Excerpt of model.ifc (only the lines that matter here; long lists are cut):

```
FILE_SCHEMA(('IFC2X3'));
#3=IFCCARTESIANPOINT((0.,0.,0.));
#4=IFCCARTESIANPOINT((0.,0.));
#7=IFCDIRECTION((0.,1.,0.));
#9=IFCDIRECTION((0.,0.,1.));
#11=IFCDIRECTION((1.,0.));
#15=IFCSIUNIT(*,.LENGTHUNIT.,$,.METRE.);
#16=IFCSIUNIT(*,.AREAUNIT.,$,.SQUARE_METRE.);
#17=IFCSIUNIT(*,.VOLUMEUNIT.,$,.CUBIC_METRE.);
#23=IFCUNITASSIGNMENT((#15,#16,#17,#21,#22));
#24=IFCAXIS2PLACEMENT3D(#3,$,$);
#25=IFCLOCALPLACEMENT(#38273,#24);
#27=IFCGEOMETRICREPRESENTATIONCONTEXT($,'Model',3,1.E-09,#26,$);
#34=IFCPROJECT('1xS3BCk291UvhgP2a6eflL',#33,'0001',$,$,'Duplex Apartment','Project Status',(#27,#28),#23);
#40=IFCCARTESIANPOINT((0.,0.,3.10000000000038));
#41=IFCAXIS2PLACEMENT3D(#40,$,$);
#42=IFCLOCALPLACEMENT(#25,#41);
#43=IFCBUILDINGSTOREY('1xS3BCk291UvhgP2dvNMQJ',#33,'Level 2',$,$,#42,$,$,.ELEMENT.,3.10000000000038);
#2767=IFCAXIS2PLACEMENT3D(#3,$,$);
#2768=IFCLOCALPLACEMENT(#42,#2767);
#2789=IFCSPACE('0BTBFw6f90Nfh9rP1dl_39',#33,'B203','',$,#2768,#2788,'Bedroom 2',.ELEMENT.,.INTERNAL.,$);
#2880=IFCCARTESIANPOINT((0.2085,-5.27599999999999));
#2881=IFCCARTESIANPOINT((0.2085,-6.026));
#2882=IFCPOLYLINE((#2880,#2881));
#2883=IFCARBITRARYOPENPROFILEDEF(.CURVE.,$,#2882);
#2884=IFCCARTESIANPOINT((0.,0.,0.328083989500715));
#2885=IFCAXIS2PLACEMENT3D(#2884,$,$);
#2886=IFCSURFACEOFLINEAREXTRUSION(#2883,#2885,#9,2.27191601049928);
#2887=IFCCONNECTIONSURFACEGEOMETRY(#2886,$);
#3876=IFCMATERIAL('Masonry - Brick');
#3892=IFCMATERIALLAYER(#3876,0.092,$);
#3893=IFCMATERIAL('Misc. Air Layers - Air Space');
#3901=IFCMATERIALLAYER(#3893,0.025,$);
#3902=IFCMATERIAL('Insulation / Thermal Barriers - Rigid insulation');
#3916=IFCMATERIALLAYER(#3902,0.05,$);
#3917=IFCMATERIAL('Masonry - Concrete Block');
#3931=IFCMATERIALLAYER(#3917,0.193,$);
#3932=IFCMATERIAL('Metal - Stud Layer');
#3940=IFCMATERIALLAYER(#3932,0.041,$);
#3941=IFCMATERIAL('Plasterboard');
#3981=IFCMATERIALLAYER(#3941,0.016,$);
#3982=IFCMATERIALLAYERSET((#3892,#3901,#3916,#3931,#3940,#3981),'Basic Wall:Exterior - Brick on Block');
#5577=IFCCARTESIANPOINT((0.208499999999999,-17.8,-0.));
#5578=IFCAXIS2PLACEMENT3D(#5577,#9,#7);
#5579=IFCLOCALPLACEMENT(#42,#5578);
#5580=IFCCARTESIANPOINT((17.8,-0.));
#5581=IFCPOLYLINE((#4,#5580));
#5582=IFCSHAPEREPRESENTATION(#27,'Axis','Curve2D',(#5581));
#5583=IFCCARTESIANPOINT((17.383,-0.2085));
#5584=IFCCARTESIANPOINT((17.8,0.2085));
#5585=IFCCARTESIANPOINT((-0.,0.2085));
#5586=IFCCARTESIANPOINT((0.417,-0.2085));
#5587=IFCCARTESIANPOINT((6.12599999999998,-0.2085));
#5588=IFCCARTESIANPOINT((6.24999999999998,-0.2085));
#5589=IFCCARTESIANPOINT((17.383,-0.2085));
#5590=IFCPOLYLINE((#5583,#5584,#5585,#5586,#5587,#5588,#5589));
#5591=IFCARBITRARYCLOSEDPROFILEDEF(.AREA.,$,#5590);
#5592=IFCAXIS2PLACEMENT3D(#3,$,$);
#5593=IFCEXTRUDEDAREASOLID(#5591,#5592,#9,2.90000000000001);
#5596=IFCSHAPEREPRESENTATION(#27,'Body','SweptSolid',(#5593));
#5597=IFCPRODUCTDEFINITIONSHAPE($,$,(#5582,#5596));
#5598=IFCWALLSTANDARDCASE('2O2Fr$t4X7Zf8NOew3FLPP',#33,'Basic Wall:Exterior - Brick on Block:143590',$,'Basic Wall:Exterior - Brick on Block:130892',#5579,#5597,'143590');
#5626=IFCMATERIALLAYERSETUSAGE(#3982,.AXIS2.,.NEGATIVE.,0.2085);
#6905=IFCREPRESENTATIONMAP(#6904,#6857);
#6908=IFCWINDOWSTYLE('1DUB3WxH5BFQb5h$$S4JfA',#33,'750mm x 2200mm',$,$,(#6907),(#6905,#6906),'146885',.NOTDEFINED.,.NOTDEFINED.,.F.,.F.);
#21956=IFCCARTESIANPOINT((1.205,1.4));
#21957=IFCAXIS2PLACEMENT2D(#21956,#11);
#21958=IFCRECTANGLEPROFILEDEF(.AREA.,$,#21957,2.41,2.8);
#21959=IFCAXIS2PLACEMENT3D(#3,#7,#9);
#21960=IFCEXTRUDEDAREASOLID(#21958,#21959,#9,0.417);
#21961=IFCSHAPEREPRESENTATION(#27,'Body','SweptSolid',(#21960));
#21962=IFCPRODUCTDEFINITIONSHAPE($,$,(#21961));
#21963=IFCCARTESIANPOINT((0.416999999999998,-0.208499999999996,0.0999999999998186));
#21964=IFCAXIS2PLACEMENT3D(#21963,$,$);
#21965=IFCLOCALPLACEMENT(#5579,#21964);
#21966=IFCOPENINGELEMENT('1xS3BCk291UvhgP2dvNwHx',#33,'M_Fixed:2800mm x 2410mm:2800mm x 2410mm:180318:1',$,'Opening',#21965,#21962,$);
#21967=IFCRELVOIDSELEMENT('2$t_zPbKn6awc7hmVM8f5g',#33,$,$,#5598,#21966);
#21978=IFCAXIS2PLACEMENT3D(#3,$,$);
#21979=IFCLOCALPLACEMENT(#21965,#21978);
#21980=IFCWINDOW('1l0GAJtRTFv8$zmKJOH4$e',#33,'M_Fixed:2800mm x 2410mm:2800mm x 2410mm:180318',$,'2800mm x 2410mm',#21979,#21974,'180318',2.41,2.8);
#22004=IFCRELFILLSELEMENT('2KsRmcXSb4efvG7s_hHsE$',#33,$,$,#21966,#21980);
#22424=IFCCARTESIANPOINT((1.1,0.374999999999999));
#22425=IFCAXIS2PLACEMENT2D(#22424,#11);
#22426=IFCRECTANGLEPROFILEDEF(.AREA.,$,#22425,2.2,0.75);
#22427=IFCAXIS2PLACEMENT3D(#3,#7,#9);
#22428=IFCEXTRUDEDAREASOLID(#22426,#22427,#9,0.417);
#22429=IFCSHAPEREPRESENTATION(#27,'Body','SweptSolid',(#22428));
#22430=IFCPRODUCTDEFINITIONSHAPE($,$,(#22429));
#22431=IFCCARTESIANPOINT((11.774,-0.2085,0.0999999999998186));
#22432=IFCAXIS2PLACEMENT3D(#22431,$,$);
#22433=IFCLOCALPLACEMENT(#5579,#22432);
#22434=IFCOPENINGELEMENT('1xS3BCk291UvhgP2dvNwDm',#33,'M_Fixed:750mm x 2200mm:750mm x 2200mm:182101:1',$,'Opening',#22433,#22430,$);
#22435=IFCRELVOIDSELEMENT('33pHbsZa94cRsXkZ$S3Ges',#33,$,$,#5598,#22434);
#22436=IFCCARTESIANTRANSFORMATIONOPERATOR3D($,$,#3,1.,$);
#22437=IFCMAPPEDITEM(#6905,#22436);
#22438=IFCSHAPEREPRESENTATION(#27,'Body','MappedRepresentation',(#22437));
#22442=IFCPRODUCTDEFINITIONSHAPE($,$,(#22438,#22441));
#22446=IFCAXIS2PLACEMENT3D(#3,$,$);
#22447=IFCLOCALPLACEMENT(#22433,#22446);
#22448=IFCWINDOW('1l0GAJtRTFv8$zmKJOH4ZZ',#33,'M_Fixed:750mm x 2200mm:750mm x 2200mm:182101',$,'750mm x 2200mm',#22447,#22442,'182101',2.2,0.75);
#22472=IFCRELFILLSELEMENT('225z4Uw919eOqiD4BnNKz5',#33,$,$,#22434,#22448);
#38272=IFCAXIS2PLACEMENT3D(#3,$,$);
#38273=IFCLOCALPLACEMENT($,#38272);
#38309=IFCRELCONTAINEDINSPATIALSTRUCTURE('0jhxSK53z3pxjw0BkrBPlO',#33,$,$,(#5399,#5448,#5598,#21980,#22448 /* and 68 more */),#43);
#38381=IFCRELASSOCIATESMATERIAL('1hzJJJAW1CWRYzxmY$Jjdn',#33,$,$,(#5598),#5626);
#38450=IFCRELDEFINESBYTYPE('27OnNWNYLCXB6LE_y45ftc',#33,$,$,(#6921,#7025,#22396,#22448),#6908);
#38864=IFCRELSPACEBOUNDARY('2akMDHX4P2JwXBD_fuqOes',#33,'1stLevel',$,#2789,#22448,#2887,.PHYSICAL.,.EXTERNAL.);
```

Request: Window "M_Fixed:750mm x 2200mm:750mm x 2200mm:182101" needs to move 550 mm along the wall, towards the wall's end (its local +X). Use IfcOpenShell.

```python
import numpy as np
import ifcopenshell
import ifcopenshell.api.geometry
import ifcopenshell.util.placement

model = ifcopenshell.open("model.ifc")

window = model.by_guid("1l0GAJtRTFv8$zmKJOH4ZZ")
opening = window.FillsVoids[0].RelatingOpeningElement
wall = opening.VoidsElements[0].RelatingBuildingElement

wall_matrix = ifcopenshell.util.placement.get_local_placement(wall.ObjectPlacement)
shift = wall_matrix[:3, 0] * 0.55
before = ifcopenshell.util.placement.get_local_placement(window.ObjectPlacement)[:3, 3].copy()

# The window is placed relative to its opening, so it follows when the opening moves.
matrix = ifcopenshell.util.placement.get_local_placement(opening.ObjectPlacement)
matrix[:3, 3] += shift
ifcopenshell.api.geometry.edit_object_placement(
    model, product=opening, matrix=matrix, is_si=False, should_transform_children=True
)

# Space boundary surfaces are stored in each space's coordinates; move them too.
for rel in window.ProvidesBoundaries:
    if not rel.ConnectionGeometry:
        continue
    surface = rel.ConnectionGeometry.SurfaceOnRelatingElement
    space_matrix = ifcopenshell.util.placement.get_local_placement(rel.RelatingSpace.ObjectPlacement)
    point = np.array(surface.Position.Location.Coordinates) + space_matrix[:3, :3].T @ shift
    surface.Position = model.createIfcAxis2Placement3D(
        model.createIfcCartesianPoint(point.tolist()), surface.Position.Axis, surface.Position.RefDirection
    )

after = ifcopenshell.util.placement.get_local_placement(window.ObjectPlacement)[:3, 3]
print("window moved by", (after - before).round(3) + 0.0)

model.write("model_updated.ifc")
```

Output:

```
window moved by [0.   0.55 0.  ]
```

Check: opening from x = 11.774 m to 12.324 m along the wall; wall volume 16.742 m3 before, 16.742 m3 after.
